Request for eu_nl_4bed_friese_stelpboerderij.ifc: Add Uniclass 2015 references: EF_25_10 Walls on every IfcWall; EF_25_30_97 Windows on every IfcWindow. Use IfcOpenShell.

First a look at what the model holds.

```python
import ifcopenshell

model = ifcopenshell.open("eu_nl_4bed_friese_stelpboerderij.ifc")
print(model.schema)
print("classifications:", [c.Name for c in model.by_type("IfcClassification")])
for ifc_class in ("IfcDoor", "IfcRoof", "IfcStair", "IfcWall", "IfcWindow"):
    print(ifc_class, len(model.by_type(ifc_class)))
```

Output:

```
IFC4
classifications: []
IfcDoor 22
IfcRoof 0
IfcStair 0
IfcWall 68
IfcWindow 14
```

```python
import ifcopenshell
import ifcopenshell.api.classification

model = ifcopenshell.open("eu_nl_4bed_friese_stelpboerderij.ifc")

system = ifcopenshell.api.classification.add_classification(model, classification="Uniclass 2015")

codes = {
    "IfcWall": ("EF_25_10", "Walls"),
    "IfcWindow": ("EF_25_30_97", "Windows"),
}
for ifc_class, (code, name) in codes.items():
    products = model.by_type(ifc_class)
    ifcopenshell.api.classification.add_reference(
        model, products=products, classification=system, identification=code, name=name
    )
    print(code, len(products))

model.write("eu_nl_4bed_friese_stelpboerderij_rev.ifc")
```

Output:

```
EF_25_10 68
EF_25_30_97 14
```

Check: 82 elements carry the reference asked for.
